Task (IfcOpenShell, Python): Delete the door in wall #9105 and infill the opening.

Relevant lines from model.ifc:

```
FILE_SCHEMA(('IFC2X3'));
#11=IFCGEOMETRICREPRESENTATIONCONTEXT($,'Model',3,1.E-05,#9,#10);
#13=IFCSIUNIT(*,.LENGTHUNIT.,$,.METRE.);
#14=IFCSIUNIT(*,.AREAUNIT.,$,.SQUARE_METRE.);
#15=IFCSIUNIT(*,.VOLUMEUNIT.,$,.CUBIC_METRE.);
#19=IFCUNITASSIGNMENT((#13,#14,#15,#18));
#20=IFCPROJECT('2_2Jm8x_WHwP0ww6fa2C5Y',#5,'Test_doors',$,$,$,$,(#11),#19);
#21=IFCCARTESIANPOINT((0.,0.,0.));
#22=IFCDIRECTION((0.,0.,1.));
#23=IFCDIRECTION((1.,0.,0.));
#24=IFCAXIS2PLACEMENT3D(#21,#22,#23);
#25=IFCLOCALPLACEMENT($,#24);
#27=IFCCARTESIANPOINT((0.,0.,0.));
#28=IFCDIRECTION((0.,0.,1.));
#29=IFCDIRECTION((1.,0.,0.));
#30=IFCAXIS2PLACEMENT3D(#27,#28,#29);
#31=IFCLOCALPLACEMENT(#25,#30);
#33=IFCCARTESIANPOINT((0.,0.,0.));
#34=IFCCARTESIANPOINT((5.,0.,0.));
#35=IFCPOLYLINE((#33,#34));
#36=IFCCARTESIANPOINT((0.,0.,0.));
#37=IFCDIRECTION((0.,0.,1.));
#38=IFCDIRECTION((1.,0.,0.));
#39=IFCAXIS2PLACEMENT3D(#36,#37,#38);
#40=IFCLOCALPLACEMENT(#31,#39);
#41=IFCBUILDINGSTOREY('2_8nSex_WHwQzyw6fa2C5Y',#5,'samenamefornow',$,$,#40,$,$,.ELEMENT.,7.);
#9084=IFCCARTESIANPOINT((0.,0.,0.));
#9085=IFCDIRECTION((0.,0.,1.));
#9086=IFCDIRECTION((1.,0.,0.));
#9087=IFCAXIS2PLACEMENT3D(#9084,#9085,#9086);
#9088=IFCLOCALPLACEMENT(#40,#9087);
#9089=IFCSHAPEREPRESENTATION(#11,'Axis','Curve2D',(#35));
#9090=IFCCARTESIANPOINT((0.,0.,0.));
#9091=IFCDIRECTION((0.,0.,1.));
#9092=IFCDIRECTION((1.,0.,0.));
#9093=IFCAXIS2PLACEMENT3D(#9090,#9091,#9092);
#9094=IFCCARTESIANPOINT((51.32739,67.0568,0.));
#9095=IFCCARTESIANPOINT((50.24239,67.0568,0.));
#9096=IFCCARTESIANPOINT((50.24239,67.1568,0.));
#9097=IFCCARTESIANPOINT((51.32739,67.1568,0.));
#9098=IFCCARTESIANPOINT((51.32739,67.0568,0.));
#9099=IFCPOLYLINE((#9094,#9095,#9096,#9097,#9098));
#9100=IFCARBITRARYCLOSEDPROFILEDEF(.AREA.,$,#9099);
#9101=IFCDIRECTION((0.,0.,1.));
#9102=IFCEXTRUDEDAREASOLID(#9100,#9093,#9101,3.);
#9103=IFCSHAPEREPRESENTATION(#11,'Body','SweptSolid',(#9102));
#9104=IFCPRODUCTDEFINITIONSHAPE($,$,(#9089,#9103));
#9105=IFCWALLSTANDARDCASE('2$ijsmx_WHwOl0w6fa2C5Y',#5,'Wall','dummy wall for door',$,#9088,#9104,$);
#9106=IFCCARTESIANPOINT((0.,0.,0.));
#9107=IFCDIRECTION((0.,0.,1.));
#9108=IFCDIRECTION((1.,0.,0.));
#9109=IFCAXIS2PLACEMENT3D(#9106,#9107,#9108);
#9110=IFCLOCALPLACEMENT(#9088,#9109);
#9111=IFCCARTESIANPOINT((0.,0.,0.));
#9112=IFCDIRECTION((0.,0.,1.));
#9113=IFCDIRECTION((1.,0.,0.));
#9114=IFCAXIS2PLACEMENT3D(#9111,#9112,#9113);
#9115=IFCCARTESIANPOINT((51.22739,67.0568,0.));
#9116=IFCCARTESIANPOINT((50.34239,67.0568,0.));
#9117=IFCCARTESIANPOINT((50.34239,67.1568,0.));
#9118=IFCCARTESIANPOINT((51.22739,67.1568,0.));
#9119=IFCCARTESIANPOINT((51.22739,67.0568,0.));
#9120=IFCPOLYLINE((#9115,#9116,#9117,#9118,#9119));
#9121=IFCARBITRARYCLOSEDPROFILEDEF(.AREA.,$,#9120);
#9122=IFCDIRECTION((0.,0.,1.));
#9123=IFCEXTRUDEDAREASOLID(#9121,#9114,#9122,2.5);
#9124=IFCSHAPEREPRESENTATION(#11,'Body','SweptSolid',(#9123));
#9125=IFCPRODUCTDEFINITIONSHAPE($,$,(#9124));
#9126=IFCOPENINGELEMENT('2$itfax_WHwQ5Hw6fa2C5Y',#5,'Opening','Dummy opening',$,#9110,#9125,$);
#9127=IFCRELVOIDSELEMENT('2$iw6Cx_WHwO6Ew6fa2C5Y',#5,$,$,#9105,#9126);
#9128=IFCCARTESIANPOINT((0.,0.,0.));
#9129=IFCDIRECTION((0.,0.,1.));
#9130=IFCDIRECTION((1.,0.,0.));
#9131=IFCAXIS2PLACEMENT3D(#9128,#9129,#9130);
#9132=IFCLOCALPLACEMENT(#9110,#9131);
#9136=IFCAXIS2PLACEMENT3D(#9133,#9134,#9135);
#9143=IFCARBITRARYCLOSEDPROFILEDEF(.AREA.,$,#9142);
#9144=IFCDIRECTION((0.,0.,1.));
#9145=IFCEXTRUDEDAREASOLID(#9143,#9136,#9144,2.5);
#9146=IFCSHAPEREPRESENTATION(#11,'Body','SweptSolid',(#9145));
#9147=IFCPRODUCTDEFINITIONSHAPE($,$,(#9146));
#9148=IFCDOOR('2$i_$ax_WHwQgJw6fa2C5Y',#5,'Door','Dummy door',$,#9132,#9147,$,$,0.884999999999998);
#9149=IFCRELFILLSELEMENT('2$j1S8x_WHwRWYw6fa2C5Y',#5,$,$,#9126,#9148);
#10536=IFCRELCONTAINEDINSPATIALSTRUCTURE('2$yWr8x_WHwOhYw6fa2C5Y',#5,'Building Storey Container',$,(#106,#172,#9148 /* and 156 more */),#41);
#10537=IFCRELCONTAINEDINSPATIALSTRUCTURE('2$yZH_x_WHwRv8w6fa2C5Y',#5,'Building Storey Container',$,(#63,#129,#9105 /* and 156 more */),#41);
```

```python
import ifcopenshell
import ifcopenshell.api.feature
import ifcopenshell.api.root
import ifcopenshell.geom
import ifcopenshell.util.shape

model = ifcopenshell.open("model.ifc")
settings = ifcopenshell.geom.settings()


def volume(element):
    """Net volume in cubic metres, openings subtracted."""
    shape = ifcopenshell.geom.create_shape(settings, element)
    return ifcopenshell.util.shape.get_volume(shape.geometry)


door = model.by_guid("2$i_$ax_WHwQgJw6fa2C5Y")
opening = door.FillsVoids[0].RelatingOpeningElement
wall = opening.VoidsElements[0].RelatingBuildingElement
before = volume(wall)

ifcopenshell.api.root.remove_product(model, product=door)
ifcopenshell.api.feature.remove_feature(model, feature=opening)

after = volume(wall)

print(f"wall volume {before:.3f} -> {after:.3f} m3")

model.write("model_rev.ifc")
```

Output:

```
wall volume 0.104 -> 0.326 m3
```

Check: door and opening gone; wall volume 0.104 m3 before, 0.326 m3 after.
